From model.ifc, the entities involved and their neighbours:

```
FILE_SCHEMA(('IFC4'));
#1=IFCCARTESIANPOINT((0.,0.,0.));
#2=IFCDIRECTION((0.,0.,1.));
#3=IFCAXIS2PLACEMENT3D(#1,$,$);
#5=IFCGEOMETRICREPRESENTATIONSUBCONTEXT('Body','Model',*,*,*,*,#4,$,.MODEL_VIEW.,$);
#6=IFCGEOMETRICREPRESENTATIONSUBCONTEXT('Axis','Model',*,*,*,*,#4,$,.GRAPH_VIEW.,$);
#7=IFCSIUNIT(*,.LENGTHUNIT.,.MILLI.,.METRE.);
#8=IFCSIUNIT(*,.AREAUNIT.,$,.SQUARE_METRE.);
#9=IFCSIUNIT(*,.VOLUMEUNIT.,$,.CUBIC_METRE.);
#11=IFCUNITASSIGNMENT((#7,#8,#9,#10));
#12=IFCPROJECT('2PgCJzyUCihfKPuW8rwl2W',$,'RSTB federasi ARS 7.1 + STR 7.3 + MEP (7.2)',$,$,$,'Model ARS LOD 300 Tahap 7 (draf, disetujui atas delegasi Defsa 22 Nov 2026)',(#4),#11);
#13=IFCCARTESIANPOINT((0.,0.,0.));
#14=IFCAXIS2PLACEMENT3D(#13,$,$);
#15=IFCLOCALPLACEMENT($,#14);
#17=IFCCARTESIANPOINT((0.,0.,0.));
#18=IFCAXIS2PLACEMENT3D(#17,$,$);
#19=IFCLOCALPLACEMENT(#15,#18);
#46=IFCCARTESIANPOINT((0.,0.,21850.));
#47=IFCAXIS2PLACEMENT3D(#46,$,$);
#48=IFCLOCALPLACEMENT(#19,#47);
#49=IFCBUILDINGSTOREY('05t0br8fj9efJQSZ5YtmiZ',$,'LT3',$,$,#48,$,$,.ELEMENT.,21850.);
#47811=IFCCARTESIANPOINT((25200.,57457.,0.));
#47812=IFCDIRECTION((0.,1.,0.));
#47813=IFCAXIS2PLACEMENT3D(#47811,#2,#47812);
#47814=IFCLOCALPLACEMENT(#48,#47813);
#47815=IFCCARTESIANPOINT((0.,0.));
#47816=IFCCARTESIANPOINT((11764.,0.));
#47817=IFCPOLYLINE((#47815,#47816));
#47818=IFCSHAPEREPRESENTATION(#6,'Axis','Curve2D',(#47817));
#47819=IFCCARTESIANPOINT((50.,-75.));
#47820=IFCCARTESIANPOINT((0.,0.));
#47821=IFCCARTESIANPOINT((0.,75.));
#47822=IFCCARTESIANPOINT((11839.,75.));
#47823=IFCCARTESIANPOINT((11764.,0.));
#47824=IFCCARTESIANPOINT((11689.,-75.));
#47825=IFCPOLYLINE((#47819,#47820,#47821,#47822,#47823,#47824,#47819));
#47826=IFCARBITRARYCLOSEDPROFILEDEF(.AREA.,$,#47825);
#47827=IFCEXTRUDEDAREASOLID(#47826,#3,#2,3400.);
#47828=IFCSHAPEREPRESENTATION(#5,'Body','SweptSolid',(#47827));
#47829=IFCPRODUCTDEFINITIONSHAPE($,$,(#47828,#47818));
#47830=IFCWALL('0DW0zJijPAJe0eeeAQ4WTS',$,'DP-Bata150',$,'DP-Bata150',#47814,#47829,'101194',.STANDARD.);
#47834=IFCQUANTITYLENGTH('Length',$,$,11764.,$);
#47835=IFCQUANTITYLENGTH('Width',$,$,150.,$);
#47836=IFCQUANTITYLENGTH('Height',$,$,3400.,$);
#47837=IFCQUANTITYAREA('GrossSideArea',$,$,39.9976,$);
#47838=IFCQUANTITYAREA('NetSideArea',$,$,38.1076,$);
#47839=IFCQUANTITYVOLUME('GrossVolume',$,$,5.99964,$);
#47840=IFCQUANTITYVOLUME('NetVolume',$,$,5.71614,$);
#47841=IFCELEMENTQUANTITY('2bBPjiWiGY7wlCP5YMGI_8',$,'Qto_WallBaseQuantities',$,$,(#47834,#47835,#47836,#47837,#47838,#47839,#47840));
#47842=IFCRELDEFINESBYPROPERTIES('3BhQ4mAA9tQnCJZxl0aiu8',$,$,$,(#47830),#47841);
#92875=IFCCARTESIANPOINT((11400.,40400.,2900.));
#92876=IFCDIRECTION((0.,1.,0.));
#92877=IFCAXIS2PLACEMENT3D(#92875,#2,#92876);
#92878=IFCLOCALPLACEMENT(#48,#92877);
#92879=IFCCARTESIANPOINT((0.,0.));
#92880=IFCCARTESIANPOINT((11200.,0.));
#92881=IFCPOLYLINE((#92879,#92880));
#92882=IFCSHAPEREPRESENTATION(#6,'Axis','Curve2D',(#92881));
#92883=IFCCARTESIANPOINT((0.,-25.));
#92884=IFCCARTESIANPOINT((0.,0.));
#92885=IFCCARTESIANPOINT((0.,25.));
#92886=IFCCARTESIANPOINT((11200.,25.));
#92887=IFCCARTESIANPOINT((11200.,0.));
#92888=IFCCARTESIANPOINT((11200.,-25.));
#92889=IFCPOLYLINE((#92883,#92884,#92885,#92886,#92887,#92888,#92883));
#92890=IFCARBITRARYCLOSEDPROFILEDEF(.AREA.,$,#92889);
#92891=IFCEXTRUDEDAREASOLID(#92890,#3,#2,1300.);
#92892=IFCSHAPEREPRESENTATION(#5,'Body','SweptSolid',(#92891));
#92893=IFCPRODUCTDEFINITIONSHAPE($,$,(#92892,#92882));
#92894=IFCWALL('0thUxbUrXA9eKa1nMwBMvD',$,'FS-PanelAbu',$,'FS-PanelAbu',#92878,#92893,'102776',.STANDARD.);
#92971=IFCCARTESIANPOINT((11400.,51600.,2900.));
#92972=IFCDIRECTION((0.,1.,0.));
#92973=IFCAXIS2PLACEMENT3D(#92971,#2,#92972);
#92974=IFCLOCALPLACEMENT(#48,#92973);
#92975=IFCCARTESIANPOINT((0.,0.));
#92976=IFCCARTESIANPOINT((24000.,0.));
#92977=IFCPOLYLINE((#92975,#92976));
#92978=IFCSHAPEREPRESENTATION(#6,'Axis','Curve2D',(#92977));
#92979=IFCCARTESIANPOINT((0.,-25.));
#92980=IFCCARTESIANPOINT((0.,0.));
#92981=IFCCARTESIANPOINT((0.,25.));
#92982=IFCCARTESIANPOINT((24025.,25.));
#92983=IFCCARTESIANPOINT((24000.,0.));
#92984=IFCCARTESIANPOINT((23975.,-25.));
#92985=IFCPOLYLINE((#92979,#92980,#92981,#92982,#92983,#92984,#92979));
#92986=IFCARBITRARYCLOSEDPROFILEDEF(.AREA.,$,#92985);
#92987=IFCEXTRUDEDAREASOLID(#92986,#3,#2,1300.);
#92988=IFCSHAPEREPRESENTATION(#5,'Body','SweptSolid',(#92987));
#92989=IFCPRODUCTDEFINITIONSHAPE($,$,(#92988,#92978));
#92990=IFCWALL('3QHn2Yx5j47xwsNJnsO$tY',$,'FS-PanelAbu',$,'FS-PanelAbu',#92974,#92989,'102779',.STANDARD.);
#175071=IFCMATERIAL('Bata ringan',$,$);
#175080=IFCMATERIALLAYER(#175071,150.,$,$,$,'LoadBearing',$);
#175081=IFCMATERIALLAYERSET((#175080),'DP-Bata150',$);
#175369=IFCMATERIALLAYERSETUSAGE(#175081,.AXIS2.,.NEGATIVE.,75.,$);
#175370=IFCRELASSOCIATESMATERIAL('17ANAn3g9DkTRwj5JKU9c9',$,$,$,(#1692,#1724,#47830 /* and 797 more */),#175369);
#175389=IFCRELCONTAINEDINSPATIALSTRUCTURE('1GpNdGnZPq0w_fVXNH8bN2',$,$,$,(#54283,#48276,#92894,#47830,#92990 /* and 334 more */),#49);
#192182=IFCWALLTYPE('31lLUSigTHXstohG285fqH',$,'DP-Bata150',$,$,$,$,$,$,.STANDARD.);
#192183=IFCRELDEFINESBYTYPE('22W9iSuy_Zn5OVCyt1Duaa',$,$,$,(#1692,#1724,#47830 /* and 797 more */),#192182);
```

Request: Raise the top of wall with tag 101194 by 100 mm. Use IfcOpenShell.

```python
import ifcopenshell
import ifcopenshell.api.pset
import ifcopenshell.geom
import ifcopenshell.util.element
import ifcopenshell.util.representation
import ifcopenshell.util.shape
import ifcopenshell.util.unit

model = ifcopenshell.open("model.ifc")
unit_scale = ifcopenshell.util.unit.calculate_unit_scale(model)
area_scale = ifcopenshell.util.unit.calculate_unit_scale(model, "AREAUNIT")
volume_scale = ifcopenshell.util.unit.calculate_unit_scale(model, "VOLUMEUNIT")
settings = ifcopenshell.geom.settings()


def volume(element):
    """Net volume in cubic metres, openings subtracted."""
    shape = ifcopenshell.geom.create_shape(settings, element)
    return ifcopenshell.util.shape.get_volume(shape.geometry)


wall = model.by_guid("0DW0zJijPAJe0eeeAQ4WTS")
before = volume(wall)

body = ifcopenshell.util.representation.get_representation(wall, "Model", "Body")
solid = body.Items[0]
old_height = solid.Depth
solid.Depth += 100.0
after = volume(wall)
thickness = 0.15  # wall thickness in metres

# Update the stored height, areas and volumes.
qto = model.by_id(ifcopenshell.util.element.get_pset(wall, "Qto_WallBaseQuantities", should_inherit=False)["id"])
ifcopenshell.api.pset.edit_qto(model, qto=qto, properties={
    "Height": solid.Depth,
    "GrossSideArea": ifcopenshell.util.element.get_pset(wall, "Qto_WallBaseQuantities", "GrossSideArea") * solid.Depth / old_height,
    "NetSideArea": after / thickness / area_scale,
    "GrossVolume": ifcopenshell.util.element.get_pset(wall, "Qto_WallBaseQuantities", "GrossVolume") * solid.Depth / old_height,
    "NetVolume": after / volume_scale,
})

print(f"height {old_height:g} -> {solid.Depth:g}, volume {before:.3f} -> {after:.3f} m3")

model.write("model_updated.ifc")
```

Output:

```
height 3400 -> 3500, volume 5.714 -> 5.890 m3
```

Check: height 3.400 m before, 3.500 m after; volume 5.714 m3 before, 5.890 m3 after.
